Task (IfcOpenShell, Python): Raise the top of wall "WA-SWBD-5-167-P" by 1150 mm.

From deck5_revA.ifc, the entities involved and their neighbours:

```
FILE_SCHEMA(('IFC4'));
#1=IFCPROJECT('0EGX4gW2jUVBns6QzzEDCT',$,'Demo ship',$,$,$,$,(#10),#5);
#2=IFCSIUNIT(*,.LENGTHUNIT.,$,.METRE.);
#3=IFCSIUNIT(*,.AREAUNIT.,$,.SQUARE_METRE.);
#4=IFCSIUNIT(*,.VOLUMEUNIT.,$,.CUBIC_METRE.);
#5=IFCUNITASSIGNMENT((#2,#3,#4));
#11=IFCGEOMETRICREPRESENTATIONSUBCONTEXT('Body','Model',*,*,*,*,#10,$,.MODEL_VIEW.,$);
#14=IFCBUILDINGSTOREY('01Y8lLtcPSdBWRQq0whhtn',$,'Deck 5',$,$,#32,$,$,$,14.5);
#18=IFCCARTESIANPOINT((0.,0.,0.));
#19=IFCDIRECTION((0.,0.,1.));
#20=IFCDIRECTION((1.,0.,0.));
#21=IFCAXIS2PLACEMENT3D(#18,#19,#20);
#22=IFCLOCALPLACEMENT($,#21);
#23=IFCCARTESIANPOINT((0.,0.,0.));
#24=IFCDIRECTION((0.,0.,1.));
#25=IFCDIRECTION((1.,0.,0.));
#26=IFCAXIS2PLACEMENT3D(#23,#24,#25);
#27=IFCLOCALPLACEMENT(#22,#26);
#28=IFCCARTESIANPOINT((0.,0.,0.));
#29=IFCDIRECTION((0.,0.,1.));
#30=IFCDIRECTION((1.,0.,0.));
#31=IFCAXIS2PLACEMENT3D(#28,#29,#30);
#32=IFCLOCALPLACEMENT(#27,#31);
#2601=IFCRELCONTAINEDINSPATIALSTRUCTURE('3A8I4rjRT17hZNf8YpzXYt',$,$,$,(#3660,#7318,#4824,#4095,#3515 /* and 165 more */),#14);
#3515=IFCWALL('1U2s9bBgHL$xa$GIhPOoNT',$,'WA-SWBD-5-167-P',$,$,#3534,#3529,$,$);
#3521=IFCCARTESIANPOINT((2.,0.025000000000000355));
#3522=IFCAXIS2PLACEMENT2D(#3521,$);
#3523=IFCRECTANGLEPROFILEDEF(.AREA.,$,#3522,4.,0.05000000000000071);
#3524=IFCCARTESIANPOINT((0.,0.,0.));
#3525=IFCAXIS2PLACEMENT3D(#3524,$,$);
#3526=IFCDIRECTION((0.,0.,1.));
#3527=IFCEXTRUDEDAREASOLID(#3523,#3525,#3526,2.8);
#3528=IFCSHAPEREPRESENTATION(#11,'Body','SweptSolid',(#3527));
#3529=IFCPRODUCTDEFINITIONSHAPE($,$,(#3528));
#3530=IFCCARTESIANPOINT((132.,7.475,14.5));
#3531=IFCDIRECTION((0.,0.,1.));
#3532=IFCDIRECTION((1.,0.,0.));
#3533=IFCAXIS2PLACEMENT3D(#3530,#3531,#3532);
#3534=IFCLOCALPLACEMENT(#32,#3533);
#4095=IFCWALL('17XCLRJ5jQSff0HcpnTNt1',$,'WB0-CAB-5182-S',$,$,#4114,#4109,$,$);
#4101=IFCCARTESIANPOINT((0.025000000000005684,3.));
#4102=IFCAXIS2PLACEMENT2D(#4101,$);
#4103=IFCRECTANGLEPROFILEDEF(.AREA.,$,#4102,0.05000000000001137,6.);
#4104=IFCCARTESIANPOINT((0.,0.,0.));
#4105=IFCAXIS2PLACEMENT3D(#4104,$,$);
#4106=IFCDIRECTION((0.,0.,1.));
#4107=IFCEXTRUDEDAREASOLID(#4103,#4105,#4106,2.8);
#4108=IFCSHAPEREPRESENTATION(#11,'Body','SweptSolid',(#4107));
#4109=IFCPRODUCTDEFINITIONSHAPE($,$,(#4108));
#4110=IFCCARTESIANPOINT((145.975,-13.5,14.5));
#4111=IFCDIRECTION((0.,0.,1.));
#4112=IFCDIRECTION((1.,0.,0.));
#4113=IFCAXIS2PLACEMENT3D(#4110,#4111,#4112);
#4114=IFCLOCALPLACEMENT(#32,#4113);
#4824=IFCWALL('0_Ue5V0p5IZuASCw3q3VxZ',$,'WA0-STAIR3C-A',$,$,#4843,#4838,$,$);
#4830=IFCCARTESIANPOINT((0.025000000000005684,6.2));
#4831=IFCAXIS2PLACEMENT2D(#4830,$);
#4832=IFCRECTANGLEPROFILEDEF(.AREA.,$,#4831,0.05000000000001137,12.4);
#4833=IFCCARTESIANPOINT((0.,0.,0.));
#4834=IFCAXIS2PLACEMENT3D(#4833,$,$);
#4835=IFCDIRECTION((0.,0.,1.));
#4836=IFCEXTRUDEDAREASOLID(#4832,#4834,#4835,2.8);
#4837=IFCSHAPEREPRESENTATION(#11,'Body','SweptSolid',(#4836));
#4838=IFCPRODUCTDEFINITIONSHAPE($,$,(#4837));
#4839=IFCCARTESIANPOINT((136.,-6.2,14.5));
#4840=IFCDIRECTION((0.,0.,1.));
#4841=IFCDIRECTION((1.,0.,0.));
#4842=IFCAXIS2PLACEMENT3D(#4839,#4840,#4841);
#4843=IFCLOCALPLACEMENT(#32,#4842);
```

```python
import ifcopenshell
import ifcopenshell.geom
import ifcopenshell.util.representation
import ifcopenshell.util.shape

model = ifcopenshell.open("deck5_revA.ifc")
settings = ifcopenshell.geom.settings()


def volume(element):
    """Net volume in cubic metres, openings subtracted."""
    shape = ifcopenshell.geom.create_shape(settings, element)
    return ifcopenshell.util.shape.get_volume(shape.geometry)


wall = model.by_guid("1U2s9bBgHL$xa$GIhPOoNT")
before = volume(wall)

body = ifcopenshell.util.representation.get_representation(wall, "Model", "Body")
solid = body.Items[0]
old_height = solid.Depth
solid.Depth += 1.15
after = volume(wall)

print(f"height {old_height:g} -> {solid.Depth:g}, volume {before:.3f} -> {after:.3f} m3")

model.write("deck5_revA_rev.ifc")
```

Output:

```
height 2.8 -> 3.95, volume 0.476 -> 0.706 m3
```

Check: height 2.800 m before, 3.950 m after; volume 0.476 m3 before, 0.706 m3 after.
